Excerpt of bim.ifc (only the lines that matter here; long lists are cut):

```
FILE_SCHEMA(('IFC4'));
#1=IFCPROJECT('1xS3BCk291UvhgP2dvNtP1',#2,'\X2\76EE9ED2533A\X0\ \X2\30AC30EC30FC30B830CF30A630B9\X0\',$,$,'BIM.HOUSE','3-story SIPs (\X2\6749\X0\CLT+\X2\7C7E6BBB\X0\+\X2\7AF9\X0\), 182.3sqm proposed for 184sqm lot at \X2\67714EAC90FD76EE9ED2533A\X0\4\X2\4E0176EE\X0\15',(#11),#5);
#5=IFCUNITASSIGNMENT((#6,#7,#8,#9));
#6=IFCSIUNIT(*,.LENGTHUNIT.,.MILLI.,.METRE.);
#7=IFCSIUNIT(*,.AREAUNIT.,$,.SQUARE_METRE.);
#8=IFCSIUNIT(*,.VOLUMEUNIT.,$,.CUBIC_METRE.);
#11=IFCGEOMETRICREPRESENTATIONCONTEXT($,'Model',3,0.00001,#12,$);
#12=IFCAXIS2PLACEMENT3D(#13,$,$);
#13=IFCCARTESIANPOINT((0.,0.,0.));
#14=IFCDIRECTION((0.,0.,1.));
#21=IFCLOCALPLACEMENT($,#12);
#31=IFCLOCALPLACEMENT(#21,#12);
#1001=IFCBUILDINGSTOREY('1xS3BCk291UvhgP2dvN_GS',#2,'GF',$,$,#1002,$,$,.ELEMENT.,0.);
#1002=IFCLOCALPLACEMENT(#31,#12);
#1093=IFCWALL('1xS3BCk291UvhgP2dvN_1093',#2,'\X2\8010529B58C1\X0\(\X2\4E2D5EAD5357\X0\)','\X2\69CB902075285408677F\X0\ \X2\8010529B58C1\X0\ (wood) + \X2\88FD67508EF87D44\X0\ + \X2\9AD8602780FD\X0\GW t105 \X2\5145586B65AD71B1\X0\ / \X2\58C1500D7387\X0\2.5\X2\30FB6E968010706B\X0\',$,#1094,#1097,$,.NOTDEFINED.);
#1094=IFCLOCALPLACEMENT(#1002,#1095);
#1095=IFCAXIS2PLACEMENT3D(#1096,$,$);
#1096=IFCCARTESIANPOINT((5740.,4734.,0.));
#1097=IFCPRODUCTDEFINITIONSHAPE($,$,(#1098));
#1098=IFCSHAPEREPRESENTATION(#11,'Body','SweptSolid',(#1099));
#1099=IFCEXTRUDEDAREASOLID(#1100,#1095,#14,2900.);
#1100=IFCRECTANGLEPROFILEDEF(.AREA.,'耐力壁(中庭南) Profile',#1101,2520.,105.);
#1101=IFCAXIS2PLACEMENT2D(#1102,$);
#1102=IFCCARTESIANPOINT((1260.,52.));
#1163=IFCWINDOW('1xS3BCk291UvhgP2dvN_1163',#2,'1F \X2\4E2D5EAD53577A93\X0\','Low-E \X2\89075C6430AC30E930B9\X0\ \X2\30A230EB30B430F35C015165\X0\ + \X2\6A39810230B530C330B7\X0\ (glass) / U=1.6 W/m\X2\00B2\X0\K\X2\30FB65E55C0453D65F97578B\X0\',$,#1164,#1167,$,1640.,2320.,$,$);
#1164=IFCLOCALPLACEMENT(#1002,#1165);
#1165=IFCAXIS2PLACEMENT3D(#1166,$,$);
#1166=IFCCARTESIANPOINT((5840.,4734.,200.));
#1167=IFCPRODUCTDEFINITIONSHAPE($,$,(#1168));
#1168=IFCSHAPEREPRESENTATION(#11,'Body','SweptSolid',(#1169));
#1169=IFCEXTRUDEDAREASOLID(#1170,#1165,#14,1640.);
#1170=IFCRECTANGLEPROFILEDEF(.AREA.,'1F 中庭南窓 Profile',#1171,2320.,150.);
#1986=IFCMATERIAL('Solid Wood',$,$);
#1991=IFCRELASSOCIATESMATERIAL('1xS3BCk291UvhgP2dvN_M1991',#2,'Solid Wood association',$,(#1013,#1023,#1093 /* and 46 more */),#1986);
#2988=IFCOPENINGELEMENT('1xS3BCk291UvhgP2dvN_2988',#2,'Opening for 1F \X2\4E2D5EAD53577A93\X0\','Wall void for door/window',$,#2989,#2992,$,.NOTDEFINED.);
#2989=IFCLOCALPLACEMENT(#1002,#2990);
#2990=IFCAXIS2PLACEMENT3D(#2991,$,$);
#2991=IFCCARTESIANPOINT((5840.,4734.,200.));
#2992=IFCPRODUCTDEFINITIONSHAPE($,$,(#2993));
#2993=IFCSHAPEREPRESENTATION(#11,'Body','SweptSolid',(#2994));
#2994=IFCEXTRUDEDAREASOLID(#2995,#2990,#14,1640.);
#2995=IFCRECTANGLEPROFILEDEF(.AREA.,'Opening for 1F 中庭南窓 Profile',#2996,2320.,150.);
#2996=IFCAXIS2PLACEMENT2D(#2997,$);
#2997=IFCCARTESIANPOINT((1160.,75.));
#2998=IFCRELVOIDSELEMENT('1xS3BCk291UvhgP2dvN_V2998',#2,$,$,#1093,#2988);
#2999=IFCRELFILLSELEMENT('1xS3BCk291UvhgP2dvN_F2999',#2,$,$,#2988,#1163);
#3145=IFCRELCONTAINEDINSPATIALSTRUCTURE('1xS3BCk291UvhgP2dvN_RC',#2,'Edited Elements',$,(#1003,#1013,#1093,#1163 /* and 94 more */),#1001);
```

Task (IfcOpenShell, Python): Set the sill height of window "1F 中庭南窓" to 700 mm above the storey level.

```python
import numpy as np
import ifcopenshell
import ifcopenshell.api.geometry
import ifcopenshell.geom
import ifcopenshell.util.element
import ifcopenshell.util.placement
import ifcopenshell.util.shape
import ifcopenshell.util.unit

model = ifcopenshell.open("bim.ifc")
unit_scale = ifcopenshell.util.unit.calculate_unit_scale(model)

window = model.by_guid("1xS3BCk291UvhgP2dvN_1163")
opening = window.FillsVoids[0].RelatingOpeningElement
storey = ifcopenshell.util.element.get_container(window, ifc_class="IfcBuildingStorey")
level = ifcopenshell.util.placement.get_local_placement(storey.ObjectPlacement)[2, 3]

# The opening's origin need not be at the sill, so measure its lowest point.
shape = ifcopenshell.geom.create_shape(ifcopenshell.geom.settings(), opening)
bottom = ifcopenshell.util.shape.get_shape_bottom_elevation(shape, shape.geometry) / unit_scale
dz = level + 700.0 - bottom

shift = np.array([0.0, 0.0, dz])
# The window is not placed relative to its opening, so move both.
for product in (opening, window):
    matrix = ifcopenshell.util.placement.get_local_placement(product.ObjectPlacement)
    matrix[:3, 3] += shift
    ifcopenshell.api.geometry.edit_object_placement(model, product=product, matrix=matrix, is_si=False)

print(f"moved by {dz * unit_scale:+.3f} m")

model.write("bim-out.ifc")
```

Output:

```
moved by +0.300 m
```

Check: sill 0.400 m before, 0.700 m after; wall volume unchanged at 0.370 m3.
